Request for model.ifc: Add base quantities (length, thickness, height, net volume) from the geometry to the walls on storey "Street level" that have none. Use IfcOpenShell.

First a look at what the model holds.

```python
import ifcopenshell
import ifcopenshell.util.element
import ifcopenshell.util.unit

model = ifcopenshell.open("model.ifc")
print(model.schema)
for unit_type in ("LENGTHUNIT", "AREAUNIT", "VOLUMEUNIT"):
    print(unit_type, ifcopenshell.util.unit.calculate_unit_scale(model, unit_type))
storey = next(s for s in model.by_type("IfcBuildingStorey") if s.Name == "Street level")
walls = [e for e in ifcopenshell.util.element.get_decomposition(storey) if e.is_a("IfcWall")]
for e in sorted(walls, key=lambda e: e.id()):
    print(e.id(), e.is_a(), e.Name, list(ifcopenshell.util.element.get_psets(e, qtos_only=True)), sep=" | ")
```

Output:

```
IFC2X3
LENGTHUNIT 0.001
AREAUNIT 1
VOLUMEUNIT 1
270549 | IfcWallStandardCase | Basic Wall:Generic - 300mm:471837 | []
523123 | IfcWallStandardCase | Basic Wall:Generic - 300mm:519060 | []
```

```python
import ifcopenshell
import ifcopenshell.api.pset
import ifcopenshell.geom
import ifcopenshell.util.element
import ifcopenshell.util.shape
import ifcopenshell.util.unit

model = ifcopenshell.open("model.ifc")
unit_scale = ifcopenshell.util.unit.calculate_unit_scale(model)
volume_scale = ifcopenshell.util.unit.calculate_unit_scale(model, "VOLUMEUNIT")
settings = ifcopenshell.geom.settings()

storey = next(s for s in model.by_type("IfcBuildingStorey") if s.Name == "Street level")
walls = [e for e in ifcopenshell.util.element.get_decomposition(storey) if e.is_a("IfcWall")]

for e in sorted(walls, key=lambda e: e.id()):
    if ifcopenshell.util.element.get_psets(e, qtos_only=True, should_inherit=False):
        continue
    # Geometry comes back in metres, in the element's own axes.
    shape = ifcopenshell.geom.create_shape(settings, e)
    values = {
        "Length": ifcopenshell.util.shape.get_x(shape.geometry) / unit_scale,
        "Width": ifcopenshell.util.shape.get_y(shape.geometry) / unit_scale,
        "Height": ifcopenshell.util.shape.get_z(shape.geometry) / unit_scale,
        "NetVolume": ifcopenshell.util.shape.get_volume(shape.geometry) / volume_scale,
    }
    qto = ifcopenshell.api.pset.add_qto(model, product=e, name="BaseQuantities")
    ifcopenshell.api.pset.edit_qto(model, qto=qto, properties=values)
    print(e.id(), {k: round(v, 3) for k, v in values.items()})

model.write("model_updated.ifc")
```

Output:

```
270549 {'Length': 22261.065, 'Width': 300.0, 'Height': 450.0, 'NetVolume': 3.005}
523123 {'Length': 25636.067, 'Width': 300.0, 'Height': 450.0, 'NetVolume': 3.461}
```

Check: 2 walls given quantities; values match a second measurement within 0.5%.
